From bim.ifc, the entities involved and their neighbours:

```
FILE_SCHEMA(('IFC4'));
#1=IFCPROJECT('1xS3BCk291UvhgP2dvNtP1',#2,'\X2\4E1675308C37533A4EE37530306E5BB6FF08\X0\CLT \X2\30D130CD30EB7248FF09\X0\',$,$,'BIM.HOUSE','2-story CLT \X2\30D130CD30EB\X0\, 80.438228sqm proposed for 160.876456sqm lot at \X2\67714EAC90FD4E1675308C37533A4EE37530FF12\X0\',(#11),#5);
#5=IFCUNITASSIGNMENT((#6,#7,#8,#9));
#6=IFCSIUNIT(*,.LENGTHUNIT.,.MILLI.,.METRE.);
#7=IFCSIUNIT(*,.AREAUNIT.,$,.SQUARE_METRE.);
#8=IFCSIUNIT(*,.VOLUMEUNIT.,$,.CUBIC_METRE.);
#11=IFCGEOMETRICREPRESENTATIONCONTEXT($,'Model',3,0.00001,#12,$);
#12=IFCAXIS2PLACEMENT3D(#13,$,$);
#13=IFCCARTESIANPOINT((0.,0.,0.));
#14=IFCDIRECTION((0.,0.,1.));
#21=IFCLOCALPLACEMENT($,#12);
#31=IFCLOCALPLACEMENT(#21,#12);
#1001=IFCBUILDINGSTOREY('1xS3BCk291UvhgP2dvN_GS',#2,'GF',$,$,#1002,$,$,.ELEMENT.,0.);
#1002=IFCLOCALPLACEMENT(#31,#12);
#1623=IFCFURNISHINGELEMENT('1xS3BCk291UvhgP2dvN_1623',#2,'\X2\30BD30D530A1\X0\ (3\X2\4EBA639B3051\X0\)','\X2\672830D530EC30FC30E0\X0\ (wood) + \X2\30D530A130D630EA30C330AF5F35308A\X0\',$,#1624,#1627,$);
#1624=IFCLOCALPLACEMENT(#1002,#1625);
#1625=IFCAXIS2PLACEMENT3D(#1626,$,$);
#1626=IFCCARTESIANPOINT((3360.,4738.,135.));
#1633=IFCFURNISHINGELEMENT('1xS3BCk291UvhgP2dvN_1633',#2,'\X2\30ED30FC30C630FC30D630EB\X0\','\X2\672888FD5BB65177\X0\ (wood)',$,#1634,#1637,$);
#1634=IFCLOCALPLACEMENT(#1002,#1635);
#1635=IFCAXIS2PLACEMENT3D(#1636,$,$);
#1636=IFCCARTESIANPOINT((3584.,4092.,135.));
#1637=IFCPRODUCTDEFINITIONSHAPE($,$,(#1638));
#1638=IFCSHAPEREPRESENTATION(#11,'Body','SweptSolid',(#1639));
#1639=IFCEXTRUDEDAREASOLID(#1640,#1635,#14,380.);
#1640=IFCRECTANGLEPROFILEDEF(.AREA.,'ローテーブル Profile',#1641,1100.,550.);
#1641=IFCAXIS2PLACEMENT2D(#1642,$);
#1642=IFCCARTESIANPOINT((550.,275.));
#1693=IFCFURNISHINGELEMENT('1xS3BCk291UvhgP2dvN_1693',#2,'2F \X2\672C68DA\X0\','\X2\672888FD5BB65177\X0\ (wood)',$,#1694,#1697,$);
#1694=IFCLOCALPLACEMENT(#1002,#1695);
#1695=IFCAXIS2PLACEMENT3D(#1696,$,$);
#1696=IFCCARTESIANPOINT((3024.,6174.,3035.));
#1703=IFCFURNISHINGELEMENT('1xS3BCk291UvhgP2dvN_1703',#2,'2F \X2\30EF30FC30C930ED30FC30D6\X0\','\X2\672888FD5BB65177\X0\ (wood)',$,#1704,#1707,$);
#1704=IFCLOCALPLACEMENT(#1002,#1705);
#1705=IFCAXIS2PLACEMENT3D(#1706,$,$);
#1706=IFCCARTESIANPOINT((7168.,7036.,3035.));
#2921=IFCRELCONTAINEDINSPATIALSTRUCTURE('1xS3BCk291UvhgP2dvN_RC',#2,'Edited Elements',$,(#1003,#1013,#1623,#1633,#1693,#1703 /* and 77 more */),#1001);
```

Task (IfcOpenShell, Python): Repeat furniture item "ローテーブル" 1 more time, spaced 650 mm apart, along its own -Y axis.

```python
import ifcopenshell
import ifcopenshell.api.geometry
import ifcopenshell.api.root
import ifcopenshell.util.element
import ifcopenshell.util.placement
import ifcopenshell.util.unit

model = ifcopenshell.open("bim.ifc")
unit_scale = ifcopenshell.util.unit.calculate_unit_scale(model)


def reuse_history(source, copy):
    """copy_class also copies each property set's owner history, people and application; keep the originals."""
    for rel in copy.IsDefinedBy:
        if rel.is_a("IfcRelDefinesByProperties") and (history := rel.RelatingPropertyDefinition.OwnerHistory):
            rel.RelatingPropertyDefinition.OwnerHistory = source.OwnerHistory
            ifcopenshell.util.element.remove_deep2(model, history)


source = model.by_id(1633)
base = ifcopenshell.util.placement.get_local_placement(source.ObjectPlacement)
step = -base[:3, 1] * 0.65 / unit_scale

for i in range(1, 2):
    copy = ifcopenshell.api.root.copy_class(model, product=source)
    copy.Representation = ifcopenshell.util.element.copy_deep(
        model, source.Representation, exclude=["IfcGeometricRepresentationContext", "IfcRepresentationMap"]
    )
    reuse_history(source, copy)
    matrix = base.copy()
    matrix[:3, 3] += i * step
    print("added at", matrix[:3, 3].round(3) + 0.0)
    ifcopenshell.api.geometry.edit_object_placement(model, product=copy, matrix=matrix, is_si=False)

model.write("bim_edited.ifc")
```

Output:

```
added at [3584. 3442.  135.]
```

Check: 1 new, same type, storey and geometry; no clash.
